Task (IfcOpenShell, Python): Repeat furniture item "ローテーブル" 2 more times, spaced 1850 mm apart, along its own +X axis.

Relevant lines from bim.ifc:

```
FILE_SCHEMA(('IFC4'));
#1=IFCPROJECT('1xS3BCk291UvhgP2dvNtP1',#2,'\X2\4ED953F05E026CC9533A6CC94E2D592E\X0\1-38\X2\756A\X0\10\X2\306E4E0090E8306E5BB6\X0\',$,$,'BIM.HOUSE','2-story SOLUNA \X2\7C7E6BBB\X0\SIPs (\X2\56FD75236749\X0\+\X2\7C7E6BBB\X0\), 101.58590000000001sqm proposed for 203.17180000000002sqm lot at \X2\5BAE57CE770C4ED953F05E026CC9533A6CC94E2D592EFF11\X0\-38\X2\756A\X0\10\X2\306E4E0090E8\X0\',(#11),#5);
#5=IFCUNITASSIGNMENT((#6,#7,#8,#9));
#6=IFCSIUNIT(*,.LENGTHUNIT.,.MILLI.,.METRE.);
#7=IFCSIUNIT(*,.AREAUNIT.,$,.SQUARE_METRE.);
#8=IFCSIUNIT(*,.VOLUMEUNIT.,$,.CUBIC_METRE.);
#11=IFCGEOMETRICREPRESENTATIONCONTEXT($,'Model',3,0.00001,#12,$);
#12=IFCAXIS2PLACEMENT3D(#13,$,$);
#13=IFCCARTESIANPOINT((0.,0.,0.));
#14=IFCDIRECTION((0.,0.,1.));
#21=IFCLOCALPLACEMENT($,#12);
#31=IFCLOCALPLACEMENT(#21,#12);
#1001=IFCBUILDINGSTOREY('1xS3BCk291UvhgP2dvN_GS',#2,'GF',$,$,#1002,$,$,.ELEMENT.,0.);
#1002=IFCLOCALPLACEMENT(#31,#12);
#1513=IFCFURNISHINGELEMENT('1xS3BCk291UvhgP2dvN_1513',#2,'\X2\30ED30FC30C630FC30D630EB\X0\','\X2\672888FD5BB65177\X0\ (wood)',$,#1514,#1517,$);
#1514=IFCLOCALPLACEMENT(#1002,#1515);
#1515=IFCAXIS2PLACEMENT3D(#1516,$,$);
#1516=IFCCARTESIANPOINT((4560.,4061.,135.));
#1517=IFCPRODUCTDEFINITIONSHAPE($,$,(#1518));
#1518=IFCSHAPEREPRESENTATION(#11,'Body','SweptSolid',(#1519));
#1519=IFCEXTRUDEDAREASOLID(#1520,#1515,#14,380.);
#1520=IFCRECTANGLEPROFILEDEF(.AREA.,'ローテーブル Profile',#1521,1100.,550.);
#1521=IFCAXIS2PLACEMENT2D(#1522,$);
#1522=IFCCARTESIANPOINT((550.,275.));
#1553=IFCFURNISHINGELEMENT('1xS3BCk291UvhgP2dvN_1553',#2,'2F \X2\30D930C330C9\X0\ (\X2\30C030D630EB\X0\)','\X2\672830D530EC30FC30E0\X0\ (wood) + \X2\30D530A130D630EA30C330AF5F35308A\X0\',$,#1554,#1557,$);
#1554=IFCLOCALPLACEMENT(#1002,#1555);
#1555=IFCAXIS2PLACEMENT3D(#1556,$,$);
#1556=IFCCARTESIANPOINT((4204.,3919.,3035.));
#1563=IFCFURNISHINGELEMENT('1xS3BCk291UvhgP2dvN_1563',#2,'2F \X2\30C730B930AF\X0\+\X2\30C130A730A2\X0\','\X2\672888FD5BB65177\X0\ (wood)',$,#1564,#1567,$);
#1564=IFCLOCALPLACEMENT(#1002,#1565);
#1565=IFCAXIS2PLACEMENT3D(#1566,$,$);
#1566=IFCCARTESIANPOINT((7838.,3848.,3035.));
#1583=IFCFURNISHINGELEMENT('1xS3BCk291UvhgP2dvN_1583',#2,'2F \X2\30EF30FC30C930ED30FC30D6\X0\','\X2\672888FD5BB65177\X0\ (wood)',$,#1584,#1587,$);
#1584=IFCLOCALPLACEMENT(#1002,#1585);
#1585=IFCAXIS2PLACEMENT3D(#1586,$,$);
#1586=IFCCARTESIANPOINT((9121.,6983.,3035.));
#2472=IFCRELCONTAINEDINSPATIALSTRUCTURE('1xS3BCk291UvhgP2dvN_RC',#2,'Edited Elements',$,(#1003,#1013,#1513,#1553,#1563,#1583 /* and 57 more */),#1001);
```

```python
import ifcopenshell
import ifcopenshell.api.geometry
import ifcopenshell.api.root
import ifcopenshell.util.element
import ifcopenshell.util.placement

model = ifcopenshell.open("bim.ifc")


def reuse_history(source, copy):
    """copy_class also copies each property set's owner history, people and application; keep the originals."""
    for rel in copy.IsDefinedBy:
        if rel.is_a("IfcRelDefinesByProperties") and (history := rel.RelatingPropertyDefinition.OwnerHistory):
            rel.RelatingPropertyDefinition.OwnerHistory = source.OwnerHistory
            ifcopenshell.util.element.remove_deep2(model, history)


source = model.by_guid("1xS3BCk291UvhgP2dvN_1513")
base = ifcopenshell.util.placement.get_local_placement(source.ObjectPlacement)
step = base[:3, 0] * 1850.0

for i in range(1, 3):
    copy = ifcopenshell.api.root.copy_class(model, product=source)
    copy.Representation = ifcopenshell.util.element.copy_deep(
        model, source.Representation, exclude=["IfcGeometricRepresentationContext", "IfcRepresentationMap"]
    )
    reuse_history(source, copy)
    matrix = base.copy()
    matrix[:3, 3] += i * step
    print("added at", matrix[:3, 3].round(3) + 0.0)
    ifcopenshell.api.geometry.edit_object_placement(model, product=copy, matrix=matrix, is_si=False)

model.write("bim-out.ifc")
```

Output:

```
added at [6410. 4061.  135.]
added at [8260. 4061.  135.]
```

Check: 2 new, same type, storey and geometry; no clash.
